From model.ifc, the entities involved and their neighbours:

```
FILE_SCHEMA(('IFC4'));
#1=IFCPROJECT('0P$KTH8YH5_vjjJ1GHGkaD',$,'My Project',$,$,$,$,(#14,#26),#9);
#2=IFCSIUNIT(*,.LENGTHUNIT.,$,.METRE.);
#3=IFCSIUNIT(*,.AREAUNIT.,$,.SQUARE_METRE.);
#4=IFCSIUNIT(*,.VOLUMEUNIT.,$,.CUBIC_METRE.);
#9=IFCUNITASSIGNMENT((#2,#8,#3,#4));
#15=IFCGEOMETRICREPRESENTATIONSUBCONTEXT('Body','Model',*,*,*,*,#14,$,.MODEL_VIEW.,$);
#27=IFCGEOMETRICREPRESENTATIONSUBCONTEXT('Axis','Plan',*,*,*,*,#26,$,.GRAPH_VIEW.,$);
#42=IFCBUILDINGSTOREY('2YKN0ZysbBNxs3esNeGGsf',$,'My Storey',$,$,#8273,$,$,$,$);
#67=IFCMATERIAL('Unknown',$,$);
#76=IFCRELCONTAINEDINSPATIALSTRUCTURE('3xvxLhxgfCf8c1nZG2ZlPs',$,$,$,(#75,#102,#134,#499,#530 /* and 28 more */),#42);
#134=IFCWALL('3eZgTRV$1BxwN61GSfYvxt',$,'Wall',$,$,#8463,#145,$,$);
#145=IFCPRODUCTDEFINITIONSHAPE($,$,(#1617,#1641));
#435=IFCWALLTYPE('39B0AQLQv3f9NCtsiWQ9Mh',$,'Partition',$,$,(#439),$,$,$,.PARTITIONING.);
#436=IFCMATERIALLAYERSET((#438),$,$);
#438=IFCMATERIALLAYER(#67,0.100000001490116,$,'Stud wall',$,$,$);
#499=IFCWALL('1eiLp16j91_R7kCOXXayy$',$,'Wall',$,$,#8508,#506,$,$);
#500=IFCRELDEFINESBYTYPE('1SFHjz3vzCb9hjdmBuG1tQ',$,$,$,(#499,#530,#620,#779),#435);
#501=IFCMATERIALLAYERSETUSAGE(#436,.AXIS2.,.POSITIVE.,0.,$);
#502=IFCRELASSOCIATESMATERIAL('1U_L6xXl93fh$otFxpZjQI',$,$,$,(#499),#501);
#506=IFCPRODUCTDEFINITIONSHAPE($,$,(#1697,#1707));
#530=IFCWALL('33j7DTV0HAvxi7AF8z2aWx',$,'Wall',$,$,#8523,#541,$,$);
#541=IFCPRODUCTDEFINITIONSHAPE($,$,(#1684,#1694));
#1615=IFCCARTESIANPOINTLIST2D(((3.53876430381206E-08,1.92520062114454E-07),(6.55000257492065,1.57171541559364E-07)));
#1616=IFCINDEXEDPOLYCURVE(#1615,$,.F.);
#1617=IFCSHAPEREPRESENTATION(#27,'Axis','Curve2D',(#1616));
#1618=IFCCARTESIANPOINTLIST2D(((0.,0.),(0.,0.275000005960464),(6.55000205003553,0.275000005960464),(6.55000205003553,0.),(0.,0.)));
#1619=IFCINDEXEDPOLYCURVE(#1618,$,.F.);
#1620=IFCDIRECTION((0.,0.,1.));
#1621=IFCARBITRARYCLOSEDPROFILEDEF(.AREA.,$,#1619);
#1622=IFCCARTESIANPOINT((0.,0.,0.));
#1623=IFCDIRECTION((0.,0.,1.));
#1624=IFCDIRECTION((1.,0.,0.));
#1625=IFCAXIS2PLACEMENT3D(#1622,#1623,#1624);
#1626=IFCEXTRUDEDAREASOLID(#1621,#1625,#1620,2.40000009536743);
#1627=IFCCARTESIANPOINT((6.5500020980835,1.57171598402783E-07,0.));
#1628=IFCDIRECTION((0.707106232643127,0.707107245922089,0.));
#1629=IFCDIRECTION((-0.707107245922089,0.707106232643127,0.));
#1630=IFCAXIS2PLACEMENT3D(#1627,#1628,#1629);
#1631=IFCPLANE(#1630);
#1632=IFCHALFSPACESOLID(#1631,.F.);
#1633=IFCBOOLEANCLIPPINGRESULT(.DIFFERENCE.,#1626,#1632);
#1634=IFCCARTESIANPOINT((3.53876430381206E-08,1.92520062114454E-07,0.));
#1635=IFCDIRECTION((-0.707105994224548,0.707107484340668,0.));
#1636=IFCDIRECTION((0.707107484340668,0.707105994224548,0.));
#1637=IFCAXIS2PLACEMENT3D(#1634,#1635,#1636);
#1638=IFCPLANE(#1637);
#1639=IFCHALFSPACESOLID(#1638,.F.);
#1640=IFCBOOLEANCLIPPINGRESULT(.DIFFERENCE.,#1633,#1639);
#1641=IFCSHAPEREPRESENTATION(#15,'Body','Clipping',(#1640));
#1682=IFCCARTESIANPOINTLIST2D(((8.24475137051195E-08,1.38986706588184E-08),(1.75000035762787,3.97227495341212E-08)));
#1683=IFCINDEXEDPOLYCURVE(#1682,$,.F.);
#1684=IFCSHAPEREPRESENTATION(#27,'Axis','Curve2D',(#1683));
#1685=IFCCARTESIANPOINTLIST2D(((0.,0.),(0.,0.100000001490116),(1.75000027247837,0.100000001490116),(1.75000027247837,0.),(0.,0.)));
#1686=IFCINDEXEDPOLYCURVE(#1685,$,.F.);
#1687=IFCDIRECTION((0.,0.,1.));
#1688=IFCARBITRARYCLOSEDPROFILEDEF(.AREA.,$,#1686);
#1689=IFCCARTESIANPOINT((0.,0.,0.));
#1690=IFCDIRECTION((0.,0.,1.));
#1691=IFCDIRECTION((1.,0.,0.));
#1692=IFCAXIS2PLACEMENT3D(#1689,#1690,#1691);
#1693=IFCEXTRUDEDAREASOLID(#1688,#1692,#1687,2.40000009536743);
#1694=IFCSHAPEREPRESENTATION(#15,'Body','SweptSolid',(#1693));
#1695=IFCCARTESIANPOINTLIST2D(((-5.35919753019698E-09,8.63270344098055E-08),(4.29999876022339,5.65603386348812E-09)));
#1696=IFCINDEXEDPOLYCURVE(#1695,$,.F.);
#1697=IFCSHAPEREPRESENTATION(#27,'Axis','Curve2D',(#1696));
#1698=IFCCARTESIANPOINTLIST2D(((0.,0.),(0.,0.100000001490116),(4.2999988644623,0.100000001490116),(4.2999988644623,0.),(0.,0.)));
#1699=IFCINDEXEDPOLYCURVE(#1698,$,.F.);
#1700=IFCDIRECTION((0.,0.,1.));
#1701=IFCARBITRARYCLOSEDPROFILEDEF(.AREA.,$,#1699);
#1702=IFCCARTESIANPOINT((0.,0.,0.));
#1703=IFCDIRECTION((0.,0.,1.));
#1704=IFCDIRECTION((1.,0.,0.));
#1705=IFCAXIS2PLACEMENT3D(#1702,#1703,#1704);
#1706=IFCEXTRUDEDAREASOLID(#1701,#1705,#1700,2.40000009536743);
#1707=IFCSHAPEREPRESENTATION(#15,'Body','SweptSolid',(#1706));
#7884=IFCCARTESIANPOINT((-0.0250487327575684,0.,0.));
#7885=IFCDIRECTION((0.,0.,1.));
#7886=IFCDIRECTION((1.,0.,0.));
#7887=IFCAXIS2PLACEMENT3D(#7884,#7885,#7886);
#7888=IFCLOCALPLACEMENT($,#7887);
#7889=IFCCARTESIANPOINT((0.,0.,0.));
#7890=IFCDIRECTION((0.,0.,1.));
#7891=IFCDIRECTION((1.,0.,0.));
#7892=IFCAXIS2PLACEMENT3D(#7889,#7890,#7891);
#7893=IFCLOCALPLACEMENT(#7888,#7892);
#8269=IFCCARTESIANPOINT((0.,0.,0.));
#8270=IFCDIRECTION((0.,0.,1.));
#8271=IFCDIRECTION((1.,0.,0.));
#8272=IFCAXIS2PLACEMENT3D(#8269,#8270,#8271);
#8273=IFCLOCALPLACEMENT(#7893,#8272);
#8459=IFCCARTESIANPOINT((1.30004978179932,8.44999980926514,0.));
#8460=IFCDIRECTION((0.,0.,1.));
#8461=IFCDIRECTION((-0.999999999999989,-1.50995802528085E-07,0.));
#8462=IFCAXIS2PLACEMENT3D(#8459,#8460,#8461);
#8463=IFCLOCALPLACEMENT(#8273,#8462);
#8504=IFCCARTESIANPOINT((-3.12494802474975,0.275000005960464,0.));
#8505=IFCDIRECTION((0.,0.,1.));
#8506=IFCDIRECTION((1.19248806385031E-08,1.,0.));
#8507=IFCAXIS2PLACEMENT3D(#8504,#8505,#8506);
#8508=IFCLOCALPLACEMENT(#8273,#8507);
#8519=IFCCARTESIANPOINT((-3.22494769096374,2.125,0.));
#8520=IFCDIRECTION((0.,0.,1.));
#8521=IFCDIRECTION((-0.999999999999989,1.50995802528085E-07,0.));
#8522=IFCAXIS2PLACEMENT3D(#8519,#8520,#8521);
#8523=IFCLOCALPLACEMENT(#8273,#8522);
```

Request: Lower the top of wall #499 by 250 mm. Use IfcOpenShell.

```python
import ifcopenshell
import ifcopenshell.geom
import ifcopenshell.util.representation
import ifcopenshell.util.shape
import ifcopenshell.util.unit

model = ifcopenshell.open("model.ifc")
unit_scale = ifcopenshell.util.unit.calculate_unit_scale(model)
settings = ifcopenshell.geom.settings()


def volume(element):
    """Net volume in cubic metres, openings subtracted."""
    shape = ifcopenshell.geom.create_shape(settings, element)
    return ifcopenshell.util.shape.get_volume(shape.geometry)


wall = model.by_guid("1eiLp16j91_R7kCOXXayy$")
before = volume(wall)

body = ifcopenshell.util.representation.get_representation(wall, "Model", "Body")
solid = body.Items[0]
old_height = solid.Depth
solid.Depth -= 0.25 / unit_scale
after = volume(wall)

print(f"height {old_height:g} -> {solid.Depth:g}, volume {before:.3f} -> {after:.3f} m3")

model.write("model_rev.ifc")
```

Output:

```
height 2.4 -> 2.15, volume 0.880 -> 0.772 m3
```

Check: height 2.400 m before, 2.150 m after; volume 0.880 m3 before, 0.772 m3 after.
